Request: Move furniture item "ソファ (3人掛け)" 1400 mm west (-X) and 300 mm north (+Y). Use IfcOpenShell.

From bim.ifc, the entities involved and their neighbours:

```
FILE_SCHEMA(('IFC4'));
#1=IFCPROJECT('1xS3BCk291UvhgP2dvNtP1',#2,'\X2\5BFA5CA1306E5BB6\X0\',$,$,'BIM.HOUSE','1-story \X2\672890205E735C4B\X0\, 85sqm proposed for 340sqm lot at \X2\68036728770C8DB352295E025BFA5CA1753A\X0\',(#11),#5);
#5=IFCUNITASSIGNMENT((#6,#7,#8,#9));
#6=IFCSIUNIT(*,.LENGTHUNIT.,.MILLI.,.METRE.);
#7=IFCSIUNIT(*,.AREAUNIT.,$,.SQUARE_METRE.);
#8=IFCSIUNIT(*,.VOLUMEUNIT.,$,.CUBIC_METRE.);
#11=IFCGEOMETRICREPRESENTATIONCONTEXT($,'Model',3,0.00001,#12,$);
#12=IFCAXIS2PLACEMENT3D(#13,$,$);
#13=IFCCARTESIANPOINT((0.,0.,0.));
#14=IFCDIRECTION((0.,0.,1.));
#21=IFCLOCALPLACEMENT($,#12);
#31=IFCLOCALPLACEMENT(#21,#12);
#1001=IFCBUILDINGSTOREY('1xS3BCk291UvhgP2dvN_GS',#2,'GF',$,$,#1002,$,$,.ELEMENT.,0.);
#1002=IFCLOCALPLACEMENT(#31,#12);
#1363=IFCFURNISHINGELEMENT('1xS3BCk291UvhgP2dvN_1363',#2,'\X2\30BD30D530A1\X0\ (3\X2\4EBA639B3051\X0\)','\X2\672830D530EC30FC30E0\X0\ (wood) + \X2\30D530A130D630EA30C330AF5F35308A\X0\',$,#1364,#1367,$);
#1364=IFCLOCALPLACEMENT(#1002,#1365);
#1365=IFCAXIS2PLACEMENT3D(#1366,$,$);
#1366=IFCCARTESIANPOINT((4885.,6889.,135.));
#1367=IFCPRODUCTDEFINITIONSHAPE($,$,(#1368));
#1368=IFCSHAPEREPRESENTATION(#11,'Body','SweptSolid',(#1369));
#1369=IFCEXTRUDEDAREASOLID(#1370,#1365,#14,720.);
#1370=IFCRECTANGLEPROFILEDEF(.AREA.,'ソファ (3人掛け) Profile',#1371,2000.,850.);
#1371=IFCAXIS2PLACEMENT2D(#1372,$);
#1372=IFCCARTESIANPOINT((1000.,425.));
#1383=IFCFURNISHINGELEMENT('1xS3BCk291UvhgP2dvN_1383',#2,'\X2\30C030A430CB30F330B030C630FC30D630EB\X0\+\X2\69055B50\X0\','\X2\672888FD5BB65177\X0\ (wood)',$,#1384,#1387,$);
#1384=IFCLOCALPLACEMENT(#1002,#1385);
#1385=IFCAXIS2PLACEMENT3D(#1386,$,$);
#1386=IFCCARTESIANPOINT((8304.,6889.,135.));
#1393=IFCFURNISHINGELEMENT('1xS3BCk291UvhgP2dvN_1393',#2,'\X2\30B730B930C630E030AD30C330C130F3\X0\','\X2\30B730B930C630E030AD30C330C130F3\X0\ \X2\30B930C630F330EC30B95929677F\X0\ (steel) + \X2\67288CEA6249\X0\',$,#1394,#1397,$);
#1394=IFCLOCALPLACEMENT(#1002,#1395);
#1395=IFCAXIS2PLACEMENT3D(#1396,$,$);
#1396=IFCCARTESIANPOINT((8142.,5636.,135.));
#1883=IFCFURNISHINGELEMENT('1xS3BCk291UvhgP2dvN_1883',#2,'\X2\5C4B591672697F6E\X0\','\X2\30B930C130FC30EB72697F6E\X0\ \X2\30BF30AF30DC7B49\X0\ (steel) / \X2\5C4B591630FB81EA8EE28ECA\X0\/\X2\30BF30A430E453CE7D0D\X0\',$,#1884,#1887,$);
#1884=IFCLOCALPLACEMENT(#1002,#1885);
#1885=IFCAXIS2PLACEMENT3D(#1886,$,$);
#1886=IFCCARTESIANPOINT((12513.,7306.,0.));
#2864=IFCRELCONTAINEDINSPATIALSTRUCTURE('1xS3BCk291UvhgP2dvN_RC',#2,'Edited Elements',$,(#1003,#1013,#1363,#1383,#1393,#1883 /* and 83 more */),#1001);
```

```python
import ifcopenshell
import ifcopenshell.api.geometry
import ifcopenshell.util.placement

model = ifcopenshell.open("bim.ifc")

item = model.by_guid("1xS3BCk291UvhgP2dvN_1363")
matrix = ifcopenshell.util.placement.get_local_placement(item.ObjectPlacement)
matrix[0, 3] -= 1400.0
matrix[1, 3] += 300.0
ifcopenshell.api.geometry.edit_object_placement(model, product=item, matrix=matrix, is_si=False)

print(ifcopenshell.util.placement.get_local_placement(item.ObjectPlacement).round(3) + 0.0)

model.write("bim_edited.ifc")
```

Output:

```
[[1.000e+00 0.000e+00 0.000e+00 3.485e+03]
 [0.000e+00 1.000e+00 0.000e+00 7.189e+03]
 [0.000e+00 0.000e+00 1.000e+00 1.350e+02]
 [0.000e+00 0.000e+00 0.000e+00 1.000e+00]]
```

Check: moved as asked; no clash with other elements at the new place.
